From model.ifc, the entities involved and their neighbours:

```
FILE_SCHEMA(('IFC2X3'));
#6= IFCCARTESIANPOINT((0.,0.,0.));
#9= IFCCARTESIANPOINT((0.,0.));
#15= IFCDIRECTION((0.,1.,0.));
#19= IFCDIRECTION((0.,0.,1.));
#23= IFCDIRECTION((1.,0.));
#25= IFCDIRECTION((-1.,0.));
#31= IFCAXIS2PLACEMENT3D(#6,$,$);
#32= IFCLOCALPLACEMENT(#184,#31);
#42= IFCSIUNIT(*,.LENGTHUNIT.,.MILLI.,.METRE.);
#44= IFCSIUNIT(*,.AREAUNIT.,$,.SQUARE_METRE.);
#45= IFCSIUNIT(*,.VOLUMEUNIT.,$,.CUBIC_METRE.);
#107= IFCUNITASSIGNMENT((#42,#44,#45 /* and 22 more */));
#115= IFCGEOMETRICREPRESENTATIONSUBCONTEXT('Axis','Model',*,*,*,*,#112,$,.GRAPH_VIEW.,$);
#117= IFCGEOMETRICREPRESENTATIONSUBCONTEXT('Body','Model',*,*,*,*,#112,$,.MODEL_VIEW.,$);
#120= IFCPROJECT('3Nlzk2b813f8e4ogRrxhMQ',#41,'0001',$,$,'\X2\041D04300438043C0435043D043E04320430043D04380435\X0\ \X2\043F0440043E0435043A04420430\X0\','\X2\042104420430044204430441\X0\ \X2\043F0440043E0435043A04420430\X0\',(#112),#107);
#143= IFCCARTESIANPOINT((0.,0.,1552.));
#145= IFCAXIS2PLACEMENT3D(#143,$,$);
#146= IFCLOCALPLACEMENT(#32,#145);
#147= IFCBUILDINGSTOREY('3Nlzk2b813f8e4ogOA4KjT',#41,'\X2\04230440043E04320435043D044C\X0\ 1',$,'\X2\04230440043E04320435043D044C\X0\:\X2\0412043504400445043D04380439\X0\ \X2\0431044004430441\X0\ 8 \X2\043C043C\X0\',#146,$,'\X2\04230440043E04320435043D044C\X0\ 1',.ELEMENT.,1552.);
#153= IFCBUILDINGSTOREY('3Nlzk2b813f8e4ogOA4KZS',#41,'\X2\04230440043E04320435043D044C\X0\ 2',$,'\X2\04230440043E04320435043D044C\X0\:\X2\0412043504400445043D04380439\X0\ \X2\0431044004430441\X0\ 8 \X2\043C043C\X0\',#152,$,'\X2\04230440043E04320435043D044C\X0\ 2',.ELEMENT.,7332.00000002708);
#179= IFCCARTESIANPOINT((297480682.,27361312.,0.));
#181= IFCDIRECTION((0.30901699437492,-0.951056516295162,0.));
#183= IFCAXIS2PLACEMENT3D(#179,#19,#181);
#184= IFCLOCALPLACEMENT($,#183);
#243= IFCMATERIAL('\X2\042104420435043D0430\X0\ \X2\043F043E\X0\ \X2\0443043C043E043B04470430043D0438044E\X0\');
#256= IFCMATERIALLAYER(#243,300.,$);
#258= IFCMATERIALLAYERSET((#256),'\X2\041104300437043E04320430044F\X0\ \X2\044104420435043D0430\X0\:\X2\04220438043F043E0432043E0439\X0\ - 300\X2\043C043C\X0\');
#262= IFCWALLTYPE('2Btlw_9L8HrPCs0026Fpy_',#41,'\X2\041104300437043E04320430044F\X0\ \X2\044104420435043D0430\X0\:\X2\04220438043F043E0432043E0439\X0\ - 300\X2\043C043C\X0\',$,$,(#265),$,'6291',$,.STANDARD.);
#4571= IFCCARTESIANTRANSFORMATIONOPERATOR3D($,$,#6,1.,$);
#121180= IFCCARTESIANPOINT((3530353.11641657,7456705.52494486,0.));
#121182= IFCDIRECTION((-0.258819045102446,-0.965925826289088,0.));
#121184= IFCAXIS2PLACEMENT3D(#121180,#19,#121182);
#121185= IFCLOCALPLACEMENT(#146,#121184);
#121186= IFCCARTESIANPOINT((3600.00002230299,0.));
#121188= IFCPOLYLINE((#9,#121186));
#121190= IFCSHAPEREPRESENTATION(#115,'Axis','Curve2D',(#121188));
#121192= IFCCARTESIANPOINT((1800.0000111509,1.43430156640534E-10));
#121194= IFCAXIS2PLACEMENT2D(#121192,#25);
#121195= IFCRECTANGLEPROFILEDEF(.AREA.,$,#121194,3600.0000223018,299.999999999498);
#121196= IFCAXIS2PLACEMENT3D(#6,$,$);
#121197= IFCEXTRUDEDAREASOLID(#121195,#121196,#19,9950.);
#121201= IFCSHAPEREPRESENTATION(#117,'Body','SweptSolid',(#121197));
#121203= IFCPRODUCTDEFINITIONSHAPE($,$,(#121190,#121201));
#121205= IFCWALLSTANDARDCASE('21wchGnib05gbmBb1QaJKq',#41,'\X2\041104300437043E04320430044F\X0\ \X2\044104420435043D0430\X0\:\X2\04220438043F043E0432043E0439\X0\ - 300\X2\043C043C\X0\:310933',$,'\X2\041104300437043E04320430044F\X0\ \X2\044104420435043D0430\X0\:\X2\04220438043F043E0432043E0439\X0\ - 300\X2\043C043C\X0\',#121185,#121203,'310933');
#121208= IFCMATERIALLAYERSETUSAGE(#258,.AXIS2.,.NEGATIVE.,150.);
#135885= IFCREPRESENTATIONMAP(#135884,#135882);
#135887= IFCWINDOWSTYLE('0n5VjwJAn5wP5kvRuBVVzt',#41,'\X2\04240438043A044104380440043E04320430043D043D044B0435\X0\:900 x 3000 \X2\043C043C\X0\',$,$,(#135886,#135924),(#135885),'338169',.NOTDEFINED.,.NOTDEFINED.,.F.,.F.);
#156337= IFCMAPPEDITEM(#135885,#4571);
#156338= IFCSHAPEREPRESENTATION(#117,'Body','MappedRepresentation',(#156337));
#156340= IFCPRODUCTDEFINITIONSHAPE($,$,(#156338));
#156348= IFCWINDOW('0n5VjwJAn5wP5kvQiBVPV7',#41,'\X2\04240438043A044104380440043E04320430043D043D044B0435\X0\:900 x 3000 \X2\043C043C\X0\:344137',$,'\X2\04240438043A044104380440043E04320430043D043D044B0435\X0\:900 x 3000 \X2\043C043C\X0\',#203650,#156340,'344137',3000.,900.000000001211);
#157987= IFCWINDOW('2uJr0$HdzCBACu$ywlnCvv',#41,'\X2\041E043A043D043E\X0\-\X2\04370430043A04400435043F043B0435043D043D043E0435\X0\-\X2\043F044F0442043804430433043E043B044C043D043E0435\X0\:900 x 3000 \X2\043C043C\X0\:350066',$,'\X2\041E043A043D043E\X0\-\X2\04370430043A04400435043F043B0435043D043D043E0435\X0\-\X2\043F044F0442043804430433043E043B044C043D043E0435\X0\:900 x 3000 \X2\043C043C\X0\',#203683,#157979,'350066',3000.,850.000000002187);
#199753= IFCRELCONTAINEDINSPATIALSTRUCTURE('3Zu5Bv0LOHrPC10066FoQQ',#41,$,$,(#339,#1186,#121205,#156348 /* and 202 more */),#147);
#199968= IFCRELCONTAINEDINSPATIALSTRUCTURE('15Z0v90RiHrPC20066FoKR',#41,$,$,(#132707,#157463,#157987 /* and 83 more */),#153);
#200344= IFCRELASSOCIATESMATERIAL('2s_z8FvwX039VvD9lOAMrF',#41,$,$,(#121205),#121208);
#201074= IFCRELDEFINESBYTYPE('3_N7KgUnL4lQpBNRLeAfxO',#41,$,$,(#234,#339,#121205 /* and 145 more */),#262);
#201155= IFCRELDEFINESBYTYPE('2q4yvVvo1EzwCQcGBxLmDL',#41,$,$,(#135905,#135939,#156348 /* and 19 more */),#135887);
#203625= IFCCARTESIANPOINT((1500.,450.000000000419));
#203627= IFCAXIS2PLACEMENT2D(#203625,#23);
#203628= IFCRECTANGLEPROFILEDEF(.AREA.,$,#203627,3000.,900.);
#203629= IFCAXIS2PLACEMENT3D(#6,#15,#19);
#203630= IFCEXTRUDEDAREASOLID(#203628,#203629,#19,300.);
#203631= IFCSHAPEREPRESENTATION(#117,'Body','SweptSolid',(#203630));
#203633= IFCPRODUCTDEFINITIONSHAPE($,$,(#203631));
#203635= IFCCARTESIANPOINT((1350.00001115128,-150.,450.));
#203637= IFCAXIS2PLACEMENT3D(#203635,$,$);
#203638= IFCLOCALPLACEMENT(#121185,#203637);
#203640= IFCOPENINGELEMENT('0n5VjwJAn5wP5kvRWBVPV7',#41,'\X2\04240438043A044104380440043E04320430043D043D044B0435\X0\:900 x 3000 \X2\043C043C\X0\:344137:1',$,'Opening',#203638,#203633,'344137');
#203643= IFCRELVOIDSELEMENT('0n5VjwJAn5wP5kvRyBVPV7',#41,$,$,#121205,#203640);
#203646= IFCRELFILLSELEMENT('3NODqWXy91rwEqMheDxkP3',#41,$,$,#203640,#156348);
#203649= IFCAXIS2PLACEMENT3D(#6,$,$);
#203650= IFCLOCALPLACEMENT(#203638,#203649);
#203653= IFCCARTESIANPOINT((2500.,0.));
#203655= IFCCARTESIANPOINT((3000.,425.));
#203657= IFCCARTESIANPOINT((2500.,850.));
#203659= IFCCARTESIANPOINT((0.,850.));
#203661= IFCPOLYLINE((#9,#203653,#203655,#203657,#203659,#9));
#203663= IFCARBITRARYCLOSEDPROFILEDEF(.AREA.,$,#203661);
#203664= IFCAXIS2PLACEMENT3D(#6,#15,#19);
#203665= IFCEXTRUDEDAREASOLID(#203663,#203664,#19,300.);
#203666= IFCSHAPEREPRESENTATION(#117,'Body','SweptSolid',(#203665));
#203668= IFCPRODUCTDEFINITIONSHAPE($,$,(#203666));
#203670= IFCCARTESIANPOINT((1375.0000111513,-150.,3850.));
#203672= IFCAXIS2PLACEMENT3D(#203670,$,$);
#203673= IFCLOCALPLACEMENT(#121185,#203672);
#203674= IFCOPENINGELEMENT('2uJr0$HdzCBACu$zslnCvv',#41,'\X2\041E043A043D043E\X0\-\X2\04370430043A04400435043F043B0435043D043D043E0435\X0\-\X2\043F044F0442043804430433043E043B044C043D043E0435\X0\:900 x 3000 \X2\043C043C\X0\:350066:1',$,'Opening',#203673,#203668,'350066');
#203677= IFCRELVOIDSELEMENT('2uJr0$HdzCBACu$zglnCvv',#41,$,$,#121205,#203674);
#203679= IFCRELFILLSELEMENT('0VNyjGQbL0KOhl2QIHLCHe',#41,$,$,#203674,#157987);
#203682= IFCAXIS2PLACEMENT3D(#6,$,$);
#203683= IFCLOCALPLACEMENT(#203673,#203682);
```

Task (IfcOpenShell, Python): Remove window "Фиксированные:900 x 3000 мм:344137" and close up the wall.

```python
import ifcopenshell
import ifcopenshell.api.feature
import ifcopenshell.api.root
import ifcopenshell.geom
import ifcopenshell.util.shape

model = ifcopenshell.open("model.ifc")
settings = ifcopenshell.geom.settings()


def volume(element):
    """Net volume in cubic metres, openings subtracted."""
    shape = ifcopenshell.geom.create_shape(settings, element)
    return ifcopenshell.util.shape.get_volume(shape.geometry)


window = model.by_guid("0n5VjwJAn5wP5kvQiBVPV7")
opening = window.FillsVoids[0].RelatingOpeningElement
wall = opening.VoidsElements[0].RelatingBuildingElement
before = volume(wall)

ifcopenshell.api.root.remove_product(model, product=window)
ifcopenshell.api.feature.remove_feature(model, feature=opening)

after = volume(wall)

print(f"wall volume {before:.3f} -> {after:.3f} m3")

model.write("model-out.ifc")
```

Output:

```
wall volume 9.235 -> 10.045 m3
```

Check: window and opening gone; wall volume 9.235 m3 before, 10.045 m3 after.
